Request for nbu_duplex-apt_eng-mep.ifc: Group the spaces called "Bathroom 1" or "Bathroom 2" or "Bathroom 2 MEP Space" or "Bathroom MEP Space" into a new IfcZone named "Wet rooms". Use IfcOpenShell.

First a look at what the model holds.

```python
import ifcopenshell

model = ifcopenshell.open("nbu_duplex-apt_eng-mep.ifc")
print(model.schema)
seen = {}
for space in model.by_type("IfcSpace"):
    seen[space.LongName] = seen.get(space.LongName, 0) + 1
for name, count in sorted(seen.items(), key=str):
    print(count, "x", name)
print("zones:", [z.Name for z in model.by_type("IfcZone")][:20])
```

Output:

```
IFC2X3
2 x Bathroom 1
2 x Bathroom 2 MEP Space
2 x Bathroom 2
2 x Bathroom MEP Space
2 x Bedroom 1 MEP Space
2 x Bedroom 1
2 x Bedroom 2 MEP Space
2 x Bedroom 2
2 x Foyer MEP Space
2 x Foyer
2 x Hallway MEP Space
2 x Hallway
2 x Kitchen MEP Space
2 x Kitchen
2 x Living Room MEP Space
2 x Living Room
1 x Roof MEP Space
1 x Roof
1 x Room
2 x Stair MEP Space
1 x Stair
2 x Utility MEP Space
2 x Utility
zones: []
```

```python
import ifcopenshell
import ifcopenshell.api.group
import ifcopenshell.api.root

model = ifcopenshell.open("nbu_duplex-apt_eng-mep.ifc")

names = {"Bathroom 1", "Bathroom 2", "Bathroom 2 MEP Space", "Bathroom MEP Space"}
spaces = [s for s in model.by_type("IfcSpace") if s.LongName in names]

zone = ifcopenshell.api.root.create_entity(model, ifc_class="IfcZone", name="Wet rooms")
ifcopenshell.api.group.assign_group(model, products=spaces, group=zone)
print(len(spaces), "spaces in", zone.Name)

model.write("nbu_duplex-apt_eng-mep_updated.ifc")
```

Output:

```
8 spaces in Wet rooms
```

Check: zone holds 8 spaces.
